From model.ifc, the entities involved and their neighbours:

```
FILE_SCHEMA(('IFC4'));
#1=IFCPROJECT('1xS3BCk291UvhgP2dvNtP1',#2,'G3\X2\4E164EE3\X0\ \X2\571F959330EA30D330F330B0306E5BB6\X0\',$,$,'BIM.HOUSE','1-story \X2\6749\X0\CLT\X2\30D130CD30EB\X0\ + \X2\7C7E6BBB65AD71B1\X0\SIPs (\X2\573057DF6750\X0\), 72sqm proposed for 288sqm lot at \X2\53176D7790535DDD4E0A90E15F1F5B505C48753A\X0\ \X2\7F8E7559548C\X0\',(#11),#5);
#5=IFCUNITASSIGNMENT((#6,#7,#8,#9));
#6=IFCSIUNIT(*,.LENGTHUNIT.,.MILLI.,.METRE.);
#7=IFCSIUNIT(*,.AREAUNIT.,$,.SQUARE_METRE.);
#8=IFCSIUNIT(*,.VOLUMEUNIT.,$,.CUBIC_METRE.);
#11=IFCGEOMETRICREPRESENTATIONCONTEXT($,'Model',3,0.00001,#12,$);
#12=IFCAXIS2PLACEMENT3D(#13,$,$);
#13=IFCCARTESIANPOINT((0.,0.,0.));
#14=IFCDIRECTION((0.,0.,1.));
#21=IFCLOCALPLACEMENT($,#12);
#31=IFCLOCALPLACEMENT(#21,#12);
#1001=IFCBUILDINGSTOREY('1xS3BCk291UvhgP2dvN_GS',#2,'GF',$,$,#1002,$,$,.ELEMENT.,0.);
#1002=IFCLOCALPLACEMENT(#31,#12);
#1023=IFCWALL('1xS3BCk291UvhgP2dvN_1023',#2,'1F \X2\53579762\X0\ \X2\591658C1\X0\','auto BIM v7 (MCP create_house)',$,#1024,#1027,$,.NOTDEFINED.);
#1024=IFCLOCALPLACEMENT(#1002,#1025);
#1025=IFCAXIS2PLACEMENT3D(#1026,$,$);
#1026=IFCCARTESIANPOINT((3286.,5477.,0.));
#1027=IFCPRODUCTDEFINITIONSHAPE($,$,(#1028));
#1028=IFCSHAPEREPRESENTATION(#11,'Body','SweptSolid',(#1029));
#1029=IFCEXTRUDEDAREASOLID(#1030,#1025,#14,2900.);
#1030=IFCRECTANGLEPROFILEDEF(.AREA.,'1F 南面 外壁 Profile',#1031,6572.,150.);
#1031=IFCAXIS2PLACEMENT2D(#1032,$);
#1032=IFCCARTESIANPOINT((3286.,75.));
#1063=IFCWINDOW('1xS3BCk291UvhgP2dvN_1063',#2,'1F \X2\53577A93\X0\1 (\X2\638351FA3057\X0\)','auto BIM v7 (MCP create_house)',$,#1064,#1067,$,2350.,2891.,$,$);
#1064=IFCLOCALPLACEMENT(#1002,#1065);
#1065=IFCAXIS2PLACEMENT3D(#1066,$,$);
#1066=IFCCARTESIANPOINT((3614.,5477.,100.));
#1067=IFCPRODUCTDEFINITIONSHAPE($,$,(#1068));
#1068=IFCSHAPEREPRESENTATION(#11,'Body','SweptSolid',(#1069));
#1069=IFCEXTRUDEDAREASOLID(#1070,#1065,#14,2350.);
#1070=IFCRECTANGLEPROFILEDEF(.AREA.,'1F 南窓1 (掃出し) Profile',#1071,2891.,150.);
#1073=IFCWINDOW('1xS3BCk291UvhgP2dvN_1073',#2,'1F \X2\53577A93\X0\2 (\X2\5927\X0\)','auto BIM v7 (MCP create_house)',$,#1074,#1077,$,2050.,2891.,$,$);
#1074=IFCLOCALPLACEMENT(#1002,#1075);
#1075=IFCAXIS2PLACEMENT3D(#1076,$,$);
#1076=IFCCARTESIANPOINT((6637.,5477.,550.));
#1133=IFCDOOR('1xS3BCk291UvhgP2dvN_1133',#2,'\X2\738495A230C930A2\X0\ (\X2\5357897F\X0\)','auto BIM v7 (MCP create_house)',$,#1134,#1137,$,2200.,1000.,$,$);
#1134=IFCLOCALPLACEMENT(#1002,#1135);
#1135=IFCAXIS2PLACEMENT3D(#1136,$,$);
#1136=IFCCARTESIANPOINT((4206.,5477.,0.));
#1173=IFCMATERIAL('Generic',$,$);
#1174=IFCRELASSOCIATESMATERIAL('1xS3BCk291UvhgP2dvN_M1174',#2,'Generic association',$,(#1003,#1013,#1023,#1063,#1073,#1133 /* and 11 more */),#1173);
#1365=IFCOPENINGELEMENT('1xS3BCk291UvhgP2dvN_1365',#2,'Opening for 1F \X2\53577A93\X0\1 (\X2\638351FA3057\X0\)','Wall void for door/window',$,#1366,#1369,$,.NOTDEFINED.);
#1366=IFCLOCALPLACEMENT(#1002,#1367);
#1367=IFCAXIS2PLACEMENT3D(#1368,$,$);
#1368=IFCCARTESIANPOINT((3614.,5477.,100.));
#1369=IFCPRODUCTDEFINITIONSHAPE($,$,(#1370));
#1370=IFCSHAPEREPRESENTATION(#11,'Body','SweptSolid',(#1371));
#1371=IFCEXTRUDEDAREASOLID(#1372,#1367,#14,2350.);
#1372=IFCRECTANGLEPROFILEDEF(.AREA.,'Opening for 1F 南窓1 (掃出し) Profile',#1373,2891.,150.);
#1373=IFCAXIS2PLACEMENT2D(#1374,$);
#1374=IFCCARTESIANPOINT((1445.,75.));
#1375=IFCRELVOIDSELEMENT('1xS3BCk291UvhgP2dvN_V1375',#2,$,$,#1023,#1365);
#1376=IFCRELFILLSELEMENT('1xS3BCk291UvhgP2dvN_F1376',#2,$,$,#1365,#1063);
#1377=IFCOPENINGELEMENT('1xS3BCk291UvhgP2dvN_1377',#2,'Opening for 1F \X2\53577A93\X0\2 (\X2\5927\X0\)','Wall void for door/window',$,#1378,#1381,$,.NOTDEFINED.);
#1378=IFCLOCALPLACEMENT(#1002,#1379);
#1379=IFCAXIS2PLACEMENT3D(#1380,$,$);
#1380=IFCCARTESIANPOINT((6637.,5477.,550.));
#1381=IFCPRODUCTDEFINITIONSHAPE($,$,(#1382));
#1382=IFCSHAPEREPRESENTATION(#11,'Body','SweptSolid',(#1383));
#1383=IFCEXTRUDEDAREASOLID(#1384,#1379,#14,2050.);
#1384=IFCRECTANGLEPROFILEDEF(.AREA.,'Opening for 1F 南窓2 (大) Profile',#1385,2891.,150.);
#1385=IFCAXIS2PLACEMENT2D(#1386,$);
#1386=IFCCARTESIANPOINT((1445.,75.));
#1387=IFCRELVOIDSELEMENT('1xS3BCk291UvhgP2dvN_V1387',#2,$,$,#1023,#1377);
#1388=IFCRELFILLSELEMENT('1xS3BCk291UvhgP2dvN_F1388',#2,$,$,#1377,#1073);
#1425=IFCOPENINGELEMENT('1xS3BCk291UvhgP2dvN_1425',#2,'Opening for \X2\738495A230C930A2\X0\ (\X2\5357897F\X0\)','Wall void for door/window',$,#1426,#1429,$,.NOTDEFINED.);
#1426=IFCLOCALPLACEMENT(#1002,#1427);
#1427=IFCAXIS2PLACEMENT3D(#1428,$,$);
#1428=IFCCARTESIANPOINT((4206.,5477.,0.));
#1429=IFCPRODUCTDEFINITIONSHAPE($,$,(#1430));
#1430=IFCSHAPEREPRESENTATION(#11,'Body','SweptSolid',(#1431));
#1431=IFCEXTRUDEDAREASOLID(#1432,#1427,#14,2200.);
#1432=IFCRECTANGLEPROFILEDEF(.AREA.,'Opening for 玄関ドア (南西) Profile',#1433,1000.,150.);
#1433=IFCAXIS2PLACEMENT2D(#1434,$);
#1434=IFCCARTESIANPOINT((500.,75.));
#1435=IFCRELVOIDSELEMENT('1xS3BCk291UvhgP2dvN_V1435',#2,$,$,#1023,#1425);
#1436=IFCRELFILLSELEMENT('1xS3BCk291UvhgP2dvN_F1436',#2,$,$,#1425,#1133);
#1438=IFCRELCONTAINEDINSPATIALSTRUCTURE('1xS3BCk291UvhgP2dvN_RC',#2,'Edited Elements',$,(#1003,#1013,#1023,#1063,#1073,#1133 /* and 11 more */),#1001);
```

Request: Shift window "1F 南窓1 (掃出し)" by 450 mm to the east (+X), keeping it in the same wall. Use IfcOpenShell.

```python
import ifcopenshell
import ifcopenshell.api.geometry
import ifcopenshell.util.placement

model = ifcopenshell.open("model.ifc")

window = model.by_id(1063)
opening = window.FillsVoids[0].RelatingOpeningElement
wall = opening.VoidsElements[0].RelatingBuildingElement

wall_matrix = ifcopenshell.util.placement.get_local_placement(wall.ObjectPlacement)
shift = wall_matrix[:3, 0] * 450.0
before = ifcopenshell.util.placement.get_local_placement(window.ObjectPlacement)[:3, 3].copy()

# The window is not placed relative to its opening, so move both.
for product in (opening, window):
    matrix = ifcopenshell.util.placement.get_local_placement(product.ObjectPlacement)
    matrix[:3, 3] += shift
    ifcopenshell.api.geometry.edit_object_placement(model, product=product, matrix=matrix, is_si=False)

after = ifcopenshell.util.placement.get_local_placement(window.ObjectPlacement)[:3, 3]
print("window moved by", (after - before).round(3) + 0.0)

model.write("model-out.ifc")
```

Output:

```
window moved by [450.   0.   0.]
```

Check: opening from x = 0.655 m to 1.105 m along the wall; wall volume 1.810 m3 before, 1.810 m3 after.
